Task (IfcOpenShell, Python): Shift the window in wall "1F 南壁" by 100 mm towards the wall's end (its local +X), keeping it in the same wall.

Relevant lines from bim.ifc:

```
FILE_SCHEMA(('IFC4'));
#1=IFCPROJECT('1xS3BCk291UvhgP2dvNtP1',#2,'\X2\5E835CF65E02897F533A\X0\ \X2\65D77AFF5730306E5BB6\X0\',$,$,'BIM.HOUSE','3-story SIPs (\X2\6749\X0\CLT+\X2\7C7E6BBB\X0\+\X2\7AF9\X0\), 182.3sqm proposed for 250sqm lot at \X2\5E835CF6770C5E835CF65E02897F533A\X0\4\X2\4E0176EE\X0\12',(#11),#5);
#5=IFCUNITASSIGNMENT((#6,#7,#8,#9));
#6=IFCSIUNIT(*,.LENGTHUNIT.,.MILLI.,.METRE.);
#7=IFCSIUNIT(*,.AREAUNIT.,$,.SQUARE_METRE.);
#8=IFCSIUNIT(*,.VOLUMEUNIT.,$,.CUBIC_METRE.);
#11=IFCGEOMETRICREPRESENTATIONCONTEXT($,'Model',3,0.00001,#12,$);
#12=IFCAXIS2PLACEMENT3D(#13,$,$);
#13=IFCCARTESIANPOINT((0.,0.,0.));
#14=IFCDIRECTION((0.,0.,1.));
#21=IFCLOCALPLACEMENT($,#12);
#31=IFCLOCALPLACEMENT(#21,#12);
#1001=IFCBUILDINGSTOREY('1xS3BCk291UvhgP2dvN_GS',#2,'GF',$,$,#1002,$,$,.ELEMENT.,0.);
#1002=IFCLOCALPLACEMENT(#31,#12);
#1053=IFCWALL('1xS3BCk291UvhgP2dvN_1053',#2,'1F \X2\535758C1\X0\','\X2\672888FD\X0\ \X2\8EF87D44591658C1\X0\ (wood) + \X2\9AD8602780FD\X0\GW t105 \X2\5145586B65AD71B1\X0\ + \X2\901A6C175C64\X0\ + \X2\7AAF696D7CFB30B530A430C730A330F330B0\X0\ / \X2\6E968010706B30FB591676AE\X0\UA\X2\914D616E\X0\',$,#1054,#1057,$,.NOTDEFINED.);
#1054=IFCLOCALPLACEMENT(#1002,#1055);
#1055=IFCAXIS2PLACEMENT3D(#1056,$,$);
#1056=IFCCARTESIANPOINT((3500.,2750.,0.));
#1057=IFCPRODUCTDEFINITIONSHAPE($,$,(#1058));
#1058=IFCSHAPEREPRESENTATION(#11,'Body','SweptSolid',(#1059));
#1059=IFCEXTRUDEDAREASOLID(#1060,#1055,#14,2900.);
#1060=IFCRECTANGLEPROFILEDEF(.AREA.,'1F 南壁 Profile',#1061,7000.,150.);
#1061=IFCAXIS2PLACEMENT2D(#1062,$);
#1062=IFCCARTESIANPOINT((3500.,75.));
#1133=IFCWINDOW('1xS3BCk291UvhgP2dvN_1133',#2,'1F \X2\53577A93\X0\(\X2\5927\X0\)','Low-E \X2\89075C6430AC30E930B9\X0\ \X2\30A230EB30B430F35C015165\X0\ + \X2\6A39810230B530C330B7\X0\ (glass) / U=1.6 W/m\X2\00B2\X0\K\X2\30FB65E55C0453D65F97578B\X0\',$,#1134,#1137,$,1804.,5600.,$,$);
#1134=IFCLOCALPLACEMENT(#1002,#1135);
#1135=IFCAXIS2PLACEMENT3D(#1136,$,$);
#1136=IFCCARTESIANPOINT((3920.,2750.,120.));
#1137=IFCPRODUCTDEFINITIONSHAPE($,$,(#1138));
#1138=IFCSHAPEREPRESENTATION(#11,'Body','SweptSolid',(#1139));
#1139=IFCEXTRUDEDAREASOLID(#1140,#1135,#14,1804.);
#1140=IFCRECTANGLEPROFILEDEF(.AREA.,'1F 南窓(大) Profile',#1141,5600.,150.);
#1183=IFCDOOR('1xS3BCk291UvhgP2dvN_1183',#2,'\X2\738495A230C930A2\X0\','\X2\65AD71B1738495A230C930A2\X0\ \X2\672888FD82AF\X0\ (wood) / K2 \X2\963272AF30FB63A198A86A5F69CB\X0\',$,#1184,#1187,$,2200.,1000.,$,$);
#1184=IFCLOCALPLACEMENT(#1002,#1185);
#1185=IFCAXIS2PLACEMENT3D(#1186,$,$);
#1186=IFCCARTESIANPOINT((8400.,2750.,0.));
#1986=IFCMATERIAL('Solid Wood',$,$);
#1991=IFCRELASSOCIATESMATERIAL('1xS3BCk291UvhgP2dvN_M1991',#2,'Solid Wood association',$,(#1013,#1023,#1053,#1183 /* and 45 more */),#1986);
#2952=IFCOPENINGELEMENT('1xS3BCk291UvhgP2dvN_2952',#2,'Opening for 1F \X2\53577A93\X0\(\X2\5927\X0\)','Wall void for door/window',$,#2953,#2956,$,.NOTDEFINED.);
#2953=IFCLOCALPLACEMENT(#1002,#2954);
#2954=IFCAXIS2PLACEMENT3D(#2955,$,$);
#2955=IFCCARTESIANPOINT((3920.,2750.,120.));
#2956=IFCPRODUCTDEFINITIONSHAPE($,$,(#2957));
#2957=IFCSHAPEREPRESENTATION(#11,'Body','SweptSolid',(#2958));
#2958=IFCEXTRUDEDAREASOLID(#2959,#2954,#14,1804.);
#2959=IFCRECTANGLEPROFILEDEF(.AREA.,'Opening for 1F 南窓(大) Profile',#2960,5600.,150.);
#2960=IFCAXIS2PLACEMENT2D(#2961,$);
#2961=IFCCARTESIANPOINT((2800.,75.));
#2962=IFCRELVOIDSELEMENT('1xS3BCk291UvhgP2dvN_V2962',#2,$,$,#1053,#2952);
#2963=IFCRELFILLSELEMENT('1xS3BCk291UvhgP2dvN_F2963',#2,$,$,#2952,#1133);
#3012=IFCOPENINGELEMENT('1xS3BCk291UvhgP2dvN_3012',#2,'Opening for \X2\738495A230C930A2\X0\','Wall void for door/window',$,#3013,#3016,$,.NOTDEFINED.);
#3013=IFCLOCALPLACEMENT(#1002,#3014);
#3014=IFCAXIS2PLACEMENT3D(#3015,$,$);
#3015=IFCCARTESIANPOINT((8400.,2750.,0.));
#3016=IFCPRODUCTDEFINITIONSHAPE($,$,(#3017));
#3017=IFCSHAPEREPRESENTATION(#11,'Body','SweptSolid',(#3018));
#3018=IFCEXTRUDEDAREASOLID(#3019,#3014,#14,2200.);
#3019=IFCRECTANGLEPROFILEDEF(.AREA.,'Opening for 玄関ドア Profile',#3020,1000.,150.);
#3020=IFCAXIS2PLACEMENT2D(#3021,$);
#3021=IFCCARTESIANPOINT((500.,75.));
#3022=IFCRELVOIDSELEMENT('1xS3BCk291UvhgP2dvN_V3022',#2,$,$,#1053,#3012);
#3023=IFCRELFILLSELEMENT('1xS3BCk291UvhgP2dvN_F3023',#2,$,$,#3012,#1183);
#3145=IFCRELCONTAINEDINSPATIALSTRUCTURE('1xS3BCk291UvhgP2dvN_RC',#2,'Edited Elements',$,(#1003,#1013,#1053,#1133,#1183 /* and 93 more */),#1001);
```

```python
import ifcopenshell
import ifcopenshell.api.geometry
import ifcopenshell.util.placement
import ifcopenshell.util.unit

model = ifcopenshell.open("bim.ifc")
unit_scale = ifcopenshell.util.unit.calculate_unit_scale(model)

window = model.by_id(1133)
opening = window.FillsVoids[0].RelatingOpeningElement
wall = opening.VoidsElements[0].RelatingBuildingElement

wall_matrix = ifcopenshell.util.placement.get_local_placement(wall.ObjectPlacement)
shift = wall_matrix[:3, 0] * 0.1 / unit_scale
before = ifcopenshell.util.placement.get_local_placement(window.ObjectPlacement)[:3, 3].copy()

# The window is not placed relative to its opening, so move both.
for product in (opening, window):
    matrix = ifcopenshell.util.placement.get_local_placement(product.ObjectPlacement)
    matrix[:3, 3] += shift
    ifcopenshell.api.geometry.edit_object_placement(model, product=product, matrix=matrix, is_si=False)

after = ifcopenshell.util.placement.get_local_placement(window.ObjectPlacement)[:3, 3]
print("window moved by", (after - before).round(3) + 0.0)

model.write("bim-out.ifc")
```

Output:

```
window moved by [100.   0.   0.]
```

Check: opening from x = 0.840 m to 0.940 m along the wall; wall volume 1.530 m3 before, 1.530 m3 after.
